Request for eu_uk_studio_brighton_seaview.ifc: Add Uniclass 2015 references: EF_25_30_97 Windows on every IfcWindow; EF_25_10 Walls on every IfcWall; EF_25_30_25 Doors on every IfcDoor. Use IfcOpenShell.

First a look at what the model holds.

```python
import ifcopenshell

model = ifcopenshell.open("eu_uk_studio_brighton_seaview.ifc")
print(model.schema)
print("classifications:", [c.Name for c in model.by_type("IfcClassification")])
for ifc_class in ("IfcDoor", "IfcRoof", "IfcStair", "IfcWall", "IfcWindow"):
    print(ifc_class, len(model.by_type(ifc_class)))
```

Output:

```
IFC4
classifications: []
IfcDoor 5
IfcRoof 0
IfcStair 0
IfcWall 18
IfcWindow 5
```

```python
import ifcopenshell
import ifcopenshell.api.classification

model = ifcopenshell.open("eu_uk_studio_brighton_seaview.ifc")

system = ifcopenshell.api.classification.add_classification(model, classification="Uniclass 2015")

codes = {
    "IfcWindow": ("EF_25_30_97", "Windows"),
    "IfcWall": ("EF_25_10", "Walls"),
    "IfcDoor": ("EF_25_30_25", "Doors"),
}
for ifc_class, (code, name) in codes.items():
    products = model.by_type(ifc_class)
    ifcopenshell.api.classification.add_reference(
        model, products=products, classification=system, identification=code, name=name
    )
    print(code, len(products))

model.write("eu_uk_studio_brighton_seaview-out.ifc")
```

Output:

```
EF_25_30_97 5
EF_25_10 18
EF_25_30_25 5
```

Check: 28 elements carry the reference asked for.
